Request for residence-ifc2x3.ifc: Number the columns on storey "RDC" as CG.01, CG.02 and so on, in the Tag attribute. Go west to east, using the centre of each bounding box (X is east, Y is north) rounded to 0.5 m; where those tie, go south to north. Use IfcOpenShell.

First a look at what the model holds.

```python
import ifcopenshell
import ifcopenshell.util.element
import ifcopenshell.util.placement

model = ifcopenshell.open("residence-ifc2x3.ifc")
print(model.schema)
storey = next(s for s in model.by_type("IfcBuildingStorey") if s.Name == "RDC")
columns = [e for e in ifcopenshell.util.element.get_decomposition(storey) if e.is_a("IfcColumn")]
for e in sorted(columns, key=lambda e: e.id()):
    origin = ifcopenshell.util.placement.get_local_placement(e.ObjectPlacement)[:3, 3]
    print(e.id(), e.Tag, e.Name, origin.round(2) + 0.0, sep=" | ")
```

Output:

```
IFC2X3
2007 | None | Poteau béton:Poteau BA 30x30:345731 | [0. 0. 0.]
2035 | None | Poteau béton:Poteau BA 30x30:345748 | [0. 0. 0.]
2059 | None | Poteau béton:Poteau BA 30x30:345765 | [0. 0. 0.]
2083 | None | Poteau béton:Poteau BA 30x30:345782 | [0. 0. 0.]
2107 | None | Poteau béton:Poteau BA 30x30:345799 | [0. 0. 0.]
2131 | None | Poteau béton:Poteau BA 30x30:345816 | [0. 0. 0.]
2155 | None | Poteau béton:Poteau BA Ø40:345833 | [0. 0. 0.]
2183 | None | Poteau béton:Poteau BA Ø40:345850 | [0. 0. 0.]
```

```python
import ifcopenshell
import ifcopenshell.geom
import ifcopenshell.util.element
import ifcopenshell.util.shape

model = ifcopenshell.open("residence-ifc2x3.ifc")
settings = ifcopenshell.geom.settings()
settings.set("use-world-coords", True)


def centre(element):
    shape = ifcopenshell.geom.create_shape(settings, element)
    return ifcopenshell.util.shape.get_bbox_centroid(shape.geometry)


storey = next(s for s in model.by_type("IfcBuildingStorey") if s.Name == "RDC")
columns = [e for e in ifcopenshell.util.element.get_decomposition(storey) if e.is_a("IfcColumn")]

# Insertion points can sit at a corner or the storey origin, so sort by the geometry (in metres).
centres = {e: centre(e) for e in columns}
columns.sort(key=lambda e: (round(centres[e][0] / 0.5), centres[e][1]))

for i, e in enumerate(columns, start=1):
    number = f"CG.{i:02d}"
    e.Tag = number
    print(e.id(), number)

model.write("residence-ifc2x3_v2.ifc")
```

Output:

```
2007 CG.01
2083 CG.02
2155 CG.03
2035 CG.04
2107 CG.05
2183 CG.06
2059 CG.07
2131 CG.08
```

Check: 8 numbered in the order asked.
